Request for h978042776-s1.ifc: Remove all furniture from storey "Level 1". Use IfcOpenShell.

First a look at what the model holds.

```python
import ifcopenshell
import ifcopenshell.util.element

model = ifcopenshell.open("h978042776-s1.ifc")
print(model.schema)
storey = next(s for s in model.by_type("IfcBuildingStorey") if s.Name == "Level 1")
furniture = [e for e in ifcopenshell.util.element.get_decomposition(storey) if e.is_a("IfcFurnishingElement")]
seen = {}
for e in furniture:
    element_type = ifcopenshell.util.element.get_type(e)
    name = element_type.Name if element_type not in (None, e) else None
    seen[name] = seen.get(name, 0) + 1
for name, count in sorted(seen.items(), key=str):
    print(count, "x", name)
```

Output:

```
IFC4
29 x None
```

```python
import ifcopenshell
import ifcopenshell.api.root
import ifcopenshell.util.element

model = ifcopenshell.open("h978042776-s1.ifc")

storey = next(s for s in model.by_type("IfcBuildingStorey") if s.Name == "Level 1")
furniture = [e for e in ifcopenshell.util.element.get_decomposition(storey) if e.is_a("IfcFurnishingElement")]

for e in furniture:
    ifcopenshell.api.root.remove_product(model, product=e)
print(len(furniture), "removed")

model.write("h978042776-s1_rev.ifc")
```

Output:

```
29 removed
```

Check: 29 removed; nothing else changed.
